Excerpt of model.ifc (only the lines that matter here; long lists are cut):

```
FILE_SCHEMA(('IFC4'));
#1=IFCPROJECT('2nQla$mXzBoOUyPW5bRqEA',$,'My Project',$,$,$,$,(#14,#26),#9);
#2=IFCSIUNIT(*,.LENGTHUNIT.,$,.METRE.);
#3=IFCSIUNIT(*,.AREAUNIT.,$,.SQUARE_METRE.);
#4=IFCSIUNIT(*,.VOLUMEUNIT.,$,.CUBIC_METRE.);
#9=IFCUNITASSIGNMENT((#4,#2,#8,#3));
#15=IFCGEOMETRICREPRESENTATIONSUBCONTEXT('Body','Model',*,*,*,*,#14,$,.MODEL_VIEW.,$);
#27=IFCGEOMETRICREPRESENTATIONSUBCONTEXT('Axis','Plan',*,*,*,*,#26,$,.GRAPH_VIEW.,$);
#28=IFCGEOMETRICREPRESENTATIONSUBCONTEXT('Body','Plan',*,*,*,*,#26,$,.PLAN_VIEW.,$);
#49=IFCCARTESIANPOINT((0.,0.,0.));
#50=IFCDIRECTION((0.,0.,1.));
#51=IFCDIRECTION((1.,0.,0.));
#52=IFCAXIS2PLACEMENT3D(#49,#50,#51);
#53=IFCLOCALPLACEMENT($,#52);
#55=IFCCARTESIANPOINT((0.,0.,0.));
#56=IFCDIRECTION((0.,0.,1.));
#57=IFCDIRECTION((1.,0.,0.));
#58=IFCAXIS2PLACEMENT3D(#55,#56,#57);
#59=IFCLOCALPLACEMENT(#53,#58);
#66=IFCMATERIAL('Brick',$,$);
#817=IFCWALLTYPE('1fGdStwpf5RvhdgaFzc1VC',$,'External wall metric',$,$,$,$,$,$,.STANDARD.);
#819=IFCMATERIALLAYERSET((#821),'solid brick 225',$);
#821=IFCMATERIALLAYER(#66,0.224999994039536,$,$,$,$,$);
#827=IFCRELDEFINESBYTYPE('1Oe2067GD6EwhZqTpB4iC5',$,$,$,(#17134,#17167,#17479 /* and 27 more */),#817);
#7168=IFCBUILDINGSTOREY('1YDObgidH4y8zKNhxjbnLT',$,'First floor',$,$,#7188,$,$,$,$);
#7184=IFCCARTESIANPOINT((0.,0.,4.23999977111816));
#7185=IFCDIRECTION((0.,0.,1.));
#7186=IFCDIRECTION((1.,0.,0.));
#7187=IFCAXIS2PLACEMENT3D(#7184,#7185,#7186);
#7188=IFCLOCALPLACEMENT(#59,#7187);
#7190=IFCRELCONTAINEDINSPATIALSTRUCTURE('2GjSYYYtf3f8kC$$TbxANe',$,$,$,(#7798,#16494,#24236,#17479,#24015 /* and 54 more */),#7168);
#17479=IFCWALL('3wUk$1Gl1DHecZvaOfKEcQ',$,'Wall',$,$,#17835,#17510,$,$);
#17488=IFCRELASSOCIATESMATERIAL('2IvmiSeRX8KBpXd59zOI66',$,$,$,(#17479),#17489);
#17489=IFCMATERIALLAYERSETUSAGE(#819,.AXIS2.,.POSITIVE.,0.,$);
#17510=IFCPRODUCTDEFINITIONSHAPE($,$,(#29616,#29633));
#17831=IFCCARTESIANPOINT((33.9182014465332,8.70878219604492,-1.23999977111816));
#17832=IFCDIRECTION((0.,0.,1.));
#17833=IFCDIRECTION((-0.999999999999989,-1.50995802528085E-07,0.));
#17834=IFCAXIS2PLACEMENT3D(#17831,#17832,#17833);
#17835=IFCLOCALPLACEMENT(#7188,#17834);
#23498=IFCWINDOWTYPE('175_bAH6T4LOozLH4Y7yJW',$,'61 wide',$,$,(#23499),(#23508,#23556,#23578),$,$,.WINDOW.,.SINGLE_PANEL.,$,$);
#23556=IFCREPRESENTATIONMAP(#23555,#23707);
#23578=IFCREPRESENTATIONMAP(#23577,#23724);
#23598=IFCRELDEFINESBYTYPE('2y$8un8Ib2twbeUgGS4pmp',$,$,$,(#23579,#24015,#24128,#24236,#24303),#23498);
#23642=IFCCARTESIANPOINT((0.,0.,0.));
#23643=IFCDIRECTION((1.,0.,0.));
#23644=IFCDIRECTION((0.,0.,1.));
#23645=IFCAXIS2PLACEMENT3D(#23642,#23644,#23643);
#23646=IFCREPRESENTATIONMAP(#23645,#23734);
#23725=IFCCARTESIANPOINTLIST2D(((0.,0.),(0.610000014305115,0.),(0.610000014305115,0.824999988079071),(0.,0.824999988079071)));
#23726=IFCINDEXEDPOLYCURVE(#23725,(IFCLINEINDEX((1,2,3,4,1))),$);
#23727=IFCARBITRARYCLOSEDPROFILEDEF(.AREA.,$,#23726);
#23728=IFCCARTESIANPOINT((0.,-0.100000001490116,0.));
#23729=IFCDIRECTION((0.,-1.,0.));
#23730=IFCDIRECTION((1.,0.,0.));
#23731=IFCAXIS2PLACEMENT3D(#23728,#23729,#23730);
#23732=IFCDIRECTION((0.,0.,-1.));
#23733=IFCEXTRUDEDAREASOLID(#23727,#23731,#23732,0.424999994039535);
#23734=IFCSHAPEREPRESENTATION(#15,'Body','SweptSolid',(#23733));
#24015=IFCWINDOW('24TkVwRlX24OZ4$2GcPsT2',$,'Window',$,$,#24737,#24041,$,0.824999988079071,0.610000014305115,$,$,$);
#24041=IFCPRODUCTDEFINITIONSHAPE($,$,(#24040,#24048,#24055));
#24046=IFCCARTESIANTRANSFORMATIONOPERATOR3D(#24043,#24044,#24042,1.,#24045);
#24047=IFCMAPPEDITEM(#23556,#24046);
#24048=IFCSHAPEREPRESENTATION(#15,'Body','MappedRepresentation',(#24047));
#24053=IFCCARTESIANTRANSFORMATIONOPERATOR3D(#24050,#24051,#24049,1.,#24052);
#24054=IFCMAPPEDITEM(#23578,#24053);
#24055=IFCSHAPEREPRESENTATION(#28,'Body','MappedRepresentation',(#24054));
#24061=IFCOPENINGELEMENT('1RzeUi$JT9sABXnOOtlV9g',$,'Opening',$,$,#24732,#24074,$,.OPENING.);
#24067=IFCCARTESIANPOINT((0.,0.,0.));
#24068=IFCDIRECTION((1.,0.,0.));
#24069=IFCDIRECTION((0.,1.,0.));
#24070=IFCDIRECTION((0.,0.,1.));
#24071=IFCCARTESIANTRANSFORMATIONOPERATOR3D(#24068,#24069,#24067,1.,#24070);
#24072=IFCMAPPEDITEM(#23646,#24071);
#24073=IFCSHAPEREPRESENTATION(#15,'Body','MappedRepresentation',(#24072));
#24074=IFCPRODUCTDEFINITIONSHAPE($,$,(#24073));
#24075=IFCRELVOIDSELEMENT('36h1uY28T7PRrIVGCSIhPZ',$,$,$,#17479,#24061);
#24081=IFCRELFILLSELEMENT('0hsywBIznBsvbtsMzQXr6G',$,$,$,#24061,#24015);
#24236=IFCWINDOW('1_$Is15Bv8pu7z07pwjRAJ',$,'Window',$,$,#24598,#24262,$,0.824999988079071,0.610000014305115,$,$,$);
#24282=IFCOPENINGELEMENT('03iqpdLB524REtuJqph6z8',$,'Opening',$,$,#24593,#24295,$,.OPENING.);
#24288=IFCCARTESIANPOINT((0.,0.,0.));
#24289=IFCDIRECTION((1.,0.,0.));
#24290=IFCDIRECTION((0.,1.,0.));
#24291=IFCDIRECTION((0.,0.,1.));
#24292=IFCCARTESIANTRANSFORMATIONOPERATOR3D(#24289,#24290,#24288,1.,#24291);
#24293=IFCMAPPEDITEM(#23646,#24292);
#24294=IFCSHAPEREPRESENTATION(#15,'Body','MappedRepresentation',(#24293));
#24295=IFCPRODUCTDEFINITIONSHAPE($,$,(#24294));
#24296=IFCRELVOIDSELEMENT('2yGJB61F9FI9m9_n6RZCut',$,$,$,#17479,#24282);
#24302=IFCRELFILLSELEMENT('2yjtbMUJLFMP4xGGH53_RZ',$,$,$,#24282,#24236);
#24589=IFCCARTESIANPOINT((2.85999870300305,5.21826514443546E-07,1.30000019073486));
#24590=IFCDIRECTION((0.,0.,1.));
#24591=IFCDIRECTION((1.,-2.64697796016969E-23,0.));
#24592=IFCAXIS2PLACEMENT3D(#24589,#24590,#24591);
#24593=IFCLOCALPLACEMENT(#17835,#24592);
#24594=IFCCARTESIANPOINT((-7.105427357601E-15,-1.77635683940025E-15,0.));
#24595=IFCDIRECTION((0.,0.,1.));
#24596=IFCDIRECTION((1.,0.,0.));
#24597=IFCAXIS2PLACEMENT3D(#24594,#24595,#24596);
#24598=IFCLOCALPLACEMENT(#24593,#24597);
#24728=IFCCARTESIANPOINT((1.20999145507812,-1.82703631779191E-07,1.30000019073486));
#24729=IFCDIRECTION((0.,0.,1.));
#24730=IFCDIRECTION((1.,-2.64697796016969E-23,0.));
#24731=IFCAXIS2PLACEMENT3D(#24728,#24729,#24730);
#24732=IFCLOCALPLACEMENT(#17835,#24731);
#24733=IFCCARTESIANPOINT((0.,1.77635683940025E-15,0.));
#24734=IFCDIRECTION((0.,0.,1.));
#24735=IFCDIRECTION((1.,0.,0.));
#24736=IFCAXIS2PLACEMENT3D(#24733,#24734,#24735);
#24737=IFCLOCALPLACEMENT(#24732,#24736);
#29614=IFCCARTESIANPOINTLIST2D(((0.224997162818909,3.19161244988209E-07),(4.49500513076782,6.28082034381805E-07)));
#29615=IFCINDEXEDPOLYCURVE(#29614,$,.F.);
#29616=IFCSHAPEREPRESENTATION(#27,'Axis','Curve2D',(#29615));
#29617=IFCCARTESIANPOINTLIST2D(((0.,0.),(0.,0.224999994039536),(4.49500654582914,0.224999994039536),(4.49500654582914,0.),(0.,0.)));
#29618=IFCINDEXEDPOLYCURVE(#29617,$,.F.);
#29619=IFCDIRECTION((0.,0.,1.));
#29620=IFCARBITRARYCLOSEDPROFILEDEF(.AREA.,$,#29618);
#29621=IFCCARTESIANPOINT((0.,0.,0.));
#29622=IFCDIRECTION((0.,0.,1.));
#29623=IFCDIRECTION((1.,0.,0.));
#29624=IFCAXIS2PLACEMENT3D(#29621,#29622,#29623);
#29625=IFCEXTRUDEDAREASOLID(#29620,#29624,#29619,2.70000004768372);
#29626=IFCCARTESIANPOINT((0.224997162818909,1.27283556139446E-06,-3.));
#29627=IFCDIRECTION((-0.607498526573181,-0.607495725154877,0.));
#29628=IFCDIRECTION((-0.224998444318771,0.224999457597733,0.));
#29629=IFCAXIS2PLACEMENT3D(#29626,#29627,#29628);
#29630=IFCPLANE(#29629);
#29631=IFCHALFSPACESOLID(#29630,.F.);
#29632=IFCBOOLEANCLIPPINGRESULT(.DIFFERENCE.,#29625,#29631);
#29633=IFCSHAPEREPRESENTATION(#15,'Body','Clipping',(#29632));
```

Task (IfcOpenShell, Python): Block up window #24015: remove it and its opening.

```python
import ifcopenshell
import ifcopenshell.api.feature
import ifcopenshell.api.root
import ifcopenshell.geom
import ifcopenshell.util.shape

model = ifcopenshell.open("model.ifc")
settings = ifcopenshell.geom.settings()


def volume(element):
    """Net volume in cubic metres, openings subtracted."""
    shape = ifcopenshell.geom.create_shape(settings, element)
    return ifcopenshell.util.shape.get_volume(shape.geometry)


window = model.by_guid("24TkVwRlX24OZ4$2GcPsT2")
opening = window.FillsVoids[0].RelatingOpeningElement
wall = opening.VoidsElements[0].RelatingBuildingElement
before = volume(wall)

ifcopenshell.api.root.remove_product(model, product=window)
ifcopenshell.api.feature.remove_feature(model, feature=opening)

after = volume(wall)

print(f"wall volume {before:.3f} -> {after:.3f} m3")

model.write("model_updated.ifc")
```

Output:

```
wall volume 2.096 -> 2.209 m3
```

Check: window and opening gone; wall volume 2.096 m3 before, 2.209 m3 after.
